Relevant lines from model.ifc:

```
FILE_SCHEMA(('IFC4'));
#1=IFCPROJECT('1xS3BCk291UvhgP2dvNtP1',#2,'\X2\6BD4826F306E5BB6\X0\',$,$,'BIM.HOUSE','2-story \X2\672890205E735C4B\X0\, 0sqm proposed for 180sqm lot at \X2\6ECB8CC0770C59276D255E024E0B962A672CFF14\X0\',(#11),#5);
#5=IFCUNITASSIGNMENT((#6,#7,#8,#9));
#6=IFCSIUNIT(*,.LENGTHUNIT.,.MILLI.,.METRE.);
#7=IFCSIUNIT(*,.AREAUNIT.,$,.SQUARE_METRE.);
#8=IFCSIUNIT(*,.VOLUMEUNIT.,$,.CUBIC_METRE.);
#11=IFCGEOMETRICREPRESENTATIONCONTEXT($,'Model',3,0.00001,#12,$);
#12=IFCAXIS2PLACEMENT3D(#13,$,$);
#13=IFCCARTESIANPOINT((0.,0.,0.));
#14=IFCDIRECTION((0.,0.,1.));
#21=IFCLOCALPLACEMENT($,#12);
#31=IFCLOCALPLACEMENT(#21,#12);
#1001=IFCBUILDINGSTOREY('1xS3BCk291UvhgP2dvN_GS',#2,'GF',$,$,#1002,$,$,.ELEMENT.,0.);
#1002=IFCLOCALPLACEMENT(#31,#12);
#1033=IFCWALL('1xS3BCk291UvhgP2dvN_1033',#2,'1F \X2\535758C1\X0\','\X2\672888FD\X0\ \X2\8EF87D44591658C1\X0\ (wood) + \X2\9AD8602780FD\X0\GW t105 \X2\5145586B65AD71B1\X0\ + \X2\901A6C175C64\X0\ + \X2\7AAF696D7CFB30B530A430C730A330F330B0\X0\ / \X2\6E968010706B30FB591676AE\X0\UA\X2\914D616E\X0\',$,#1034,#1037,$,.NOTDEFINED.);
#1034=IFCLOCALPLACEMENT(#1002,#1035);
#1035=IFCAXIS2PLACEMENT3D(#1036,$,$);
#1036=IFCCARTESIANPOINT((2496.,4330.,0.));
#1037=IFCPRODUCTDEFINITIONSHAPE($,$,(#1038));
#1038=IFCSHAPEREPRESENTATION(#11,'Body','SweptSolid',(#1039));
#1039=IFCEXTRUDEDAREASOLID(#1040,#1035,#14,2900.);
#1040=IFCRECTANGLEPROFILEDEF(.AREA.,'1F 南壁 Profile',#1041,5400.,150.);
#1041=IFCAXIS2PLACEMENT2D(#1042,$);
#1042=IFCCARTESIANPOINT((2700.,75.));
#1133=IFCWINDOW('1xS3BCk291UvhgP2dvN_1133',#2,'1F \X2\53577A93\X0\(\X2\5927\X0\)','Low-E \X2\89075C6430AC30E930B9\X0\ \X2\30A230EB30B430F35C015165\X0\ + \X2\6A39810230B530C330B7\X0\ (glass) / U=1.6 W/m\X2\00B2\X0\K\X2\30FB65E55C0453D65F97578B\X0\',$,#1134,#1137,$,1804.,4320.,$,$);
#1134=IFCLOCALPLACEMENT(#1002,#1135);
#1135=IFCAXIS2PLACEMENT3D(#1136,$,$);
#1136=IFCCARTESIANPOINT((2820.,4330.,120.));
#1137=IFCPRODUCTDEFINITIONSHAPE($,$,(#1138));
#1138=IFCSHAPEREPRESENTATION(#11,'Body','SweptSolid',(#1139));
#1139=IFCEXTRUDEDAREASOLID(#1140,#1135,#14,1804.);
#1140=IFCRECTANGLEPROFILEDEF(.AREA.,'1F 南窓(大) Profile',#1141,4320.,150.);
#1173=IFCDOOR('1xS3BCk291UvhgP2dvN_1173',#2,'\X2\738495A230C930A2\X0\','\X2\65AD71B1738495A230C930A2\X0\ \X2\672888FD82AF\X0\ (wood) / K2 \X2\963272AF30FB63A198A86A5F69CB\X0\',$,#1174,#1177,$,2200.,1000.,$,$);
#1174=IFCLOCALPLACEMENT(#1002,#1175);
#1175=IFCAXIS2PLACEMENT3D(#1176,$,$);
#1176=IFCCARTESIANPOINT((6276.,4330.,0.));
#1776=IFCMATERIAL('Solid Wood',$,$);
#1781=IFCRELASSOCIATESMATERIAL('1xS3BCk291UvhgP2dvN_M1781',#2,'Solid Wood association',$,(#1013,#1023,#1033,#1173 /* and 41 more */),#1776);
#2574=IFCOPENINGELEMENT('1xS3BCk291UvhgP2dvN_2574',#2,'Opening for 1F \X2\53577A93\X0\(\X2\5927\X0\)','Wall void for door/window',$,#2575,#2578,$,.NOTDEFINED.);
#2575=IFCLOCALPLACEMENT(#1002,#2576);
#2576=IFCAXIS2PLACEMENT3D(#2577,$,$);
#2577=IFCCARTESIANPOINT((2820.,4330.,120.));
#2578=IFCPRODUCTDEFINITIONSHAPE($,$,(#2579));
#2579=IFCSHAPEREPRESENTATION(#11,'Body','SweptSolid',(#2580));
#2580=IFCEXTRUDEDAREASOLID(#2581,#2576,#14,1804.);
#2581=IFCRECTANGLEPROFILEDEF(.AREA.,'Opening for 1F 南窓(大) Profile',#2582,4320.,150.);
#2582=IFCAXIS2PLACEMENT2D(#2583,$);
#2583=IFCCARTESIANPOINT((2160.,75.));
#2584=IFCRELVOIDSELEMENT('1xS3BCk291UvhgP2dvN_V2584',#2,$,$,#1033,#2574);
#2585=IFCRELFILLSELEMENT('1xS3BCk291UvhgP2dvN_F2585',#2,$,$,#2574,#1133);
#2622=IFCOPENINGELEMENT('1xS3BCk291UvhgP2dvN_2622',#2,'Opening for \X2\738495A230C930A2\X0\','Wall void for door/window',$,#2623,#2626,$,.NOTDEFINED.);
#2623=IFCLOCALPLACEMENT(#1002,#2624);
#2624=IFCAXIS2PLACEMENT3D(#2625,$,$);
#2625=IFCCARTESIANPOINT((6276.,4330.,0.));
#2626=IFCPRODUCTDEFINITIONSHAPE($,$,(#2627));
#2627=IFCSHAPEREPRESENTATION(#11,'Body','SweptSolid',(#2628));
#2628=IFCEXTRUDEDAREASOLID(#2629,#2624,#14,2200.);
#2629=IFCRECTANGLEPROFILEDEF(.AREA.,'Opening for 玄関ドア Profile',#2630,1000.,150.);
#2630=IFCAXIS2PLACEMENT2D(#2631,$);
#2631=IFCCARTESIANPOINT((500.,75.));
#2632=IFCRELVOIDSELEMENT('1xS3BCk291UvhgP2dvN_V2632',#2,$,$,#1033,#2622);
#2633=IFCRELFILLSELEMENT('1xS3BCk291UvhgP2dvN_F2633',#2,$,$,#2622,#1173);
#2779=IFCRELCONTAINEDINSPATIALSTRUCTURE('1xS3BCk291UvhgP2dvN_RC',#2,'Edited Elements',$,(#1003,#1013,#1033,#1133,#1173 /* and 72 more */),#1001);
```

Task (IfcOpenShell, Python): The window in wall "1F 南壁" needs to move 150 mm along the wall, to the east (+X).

```python
import ifcopenshell
import ifcopenshell.api.geometry
import ifcopenshell.util.placement
import ifcopenshell.util.unit

model = ifcopenshell.open("model.ifc")
unit_scale = ifcopenshell.util.unit.calculate_unit_scale(model)

window = model.by_guid("1xS3BCk291UvhgP2dvN_1133")
opening = window.FillsVoids[0].RelatingOpeningElement
wall = opening.VoidsElements[0].RelatingBuildingElement

wall_matrix = ifcopenshell.util.placement.get_local_placement(wall.ObjectPlacement)
shift = wall_matrix[:3, 0] * 0.15 / unit_scale
before = ifcopenshell.util.placement.get_local_placement(window.ObjectPlacement)[:3, 3].copy()

# The window is not placed relative to its opening, so move both.
for product in (opening, window):
    matrix = ifcopenshell.util.placement.get_local_placement(product.ObjectPlacement)
    matrix[:3, 3] += shift
    ifcopenshell.api.geometry.edit_object_placement(model, product=product, matrix=matrix, is_si=False)

after = ifcopenshell.util.placement.get_local_placement(window.ObjectPlacement)[:3, 3]
print("window moved by", (after - before).round(3) + 0.0)

model.write("model_v2.ifc")
```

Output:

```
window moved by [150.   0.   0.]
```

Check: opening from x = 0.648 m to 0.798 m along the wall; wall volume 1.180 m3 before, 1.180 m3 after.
